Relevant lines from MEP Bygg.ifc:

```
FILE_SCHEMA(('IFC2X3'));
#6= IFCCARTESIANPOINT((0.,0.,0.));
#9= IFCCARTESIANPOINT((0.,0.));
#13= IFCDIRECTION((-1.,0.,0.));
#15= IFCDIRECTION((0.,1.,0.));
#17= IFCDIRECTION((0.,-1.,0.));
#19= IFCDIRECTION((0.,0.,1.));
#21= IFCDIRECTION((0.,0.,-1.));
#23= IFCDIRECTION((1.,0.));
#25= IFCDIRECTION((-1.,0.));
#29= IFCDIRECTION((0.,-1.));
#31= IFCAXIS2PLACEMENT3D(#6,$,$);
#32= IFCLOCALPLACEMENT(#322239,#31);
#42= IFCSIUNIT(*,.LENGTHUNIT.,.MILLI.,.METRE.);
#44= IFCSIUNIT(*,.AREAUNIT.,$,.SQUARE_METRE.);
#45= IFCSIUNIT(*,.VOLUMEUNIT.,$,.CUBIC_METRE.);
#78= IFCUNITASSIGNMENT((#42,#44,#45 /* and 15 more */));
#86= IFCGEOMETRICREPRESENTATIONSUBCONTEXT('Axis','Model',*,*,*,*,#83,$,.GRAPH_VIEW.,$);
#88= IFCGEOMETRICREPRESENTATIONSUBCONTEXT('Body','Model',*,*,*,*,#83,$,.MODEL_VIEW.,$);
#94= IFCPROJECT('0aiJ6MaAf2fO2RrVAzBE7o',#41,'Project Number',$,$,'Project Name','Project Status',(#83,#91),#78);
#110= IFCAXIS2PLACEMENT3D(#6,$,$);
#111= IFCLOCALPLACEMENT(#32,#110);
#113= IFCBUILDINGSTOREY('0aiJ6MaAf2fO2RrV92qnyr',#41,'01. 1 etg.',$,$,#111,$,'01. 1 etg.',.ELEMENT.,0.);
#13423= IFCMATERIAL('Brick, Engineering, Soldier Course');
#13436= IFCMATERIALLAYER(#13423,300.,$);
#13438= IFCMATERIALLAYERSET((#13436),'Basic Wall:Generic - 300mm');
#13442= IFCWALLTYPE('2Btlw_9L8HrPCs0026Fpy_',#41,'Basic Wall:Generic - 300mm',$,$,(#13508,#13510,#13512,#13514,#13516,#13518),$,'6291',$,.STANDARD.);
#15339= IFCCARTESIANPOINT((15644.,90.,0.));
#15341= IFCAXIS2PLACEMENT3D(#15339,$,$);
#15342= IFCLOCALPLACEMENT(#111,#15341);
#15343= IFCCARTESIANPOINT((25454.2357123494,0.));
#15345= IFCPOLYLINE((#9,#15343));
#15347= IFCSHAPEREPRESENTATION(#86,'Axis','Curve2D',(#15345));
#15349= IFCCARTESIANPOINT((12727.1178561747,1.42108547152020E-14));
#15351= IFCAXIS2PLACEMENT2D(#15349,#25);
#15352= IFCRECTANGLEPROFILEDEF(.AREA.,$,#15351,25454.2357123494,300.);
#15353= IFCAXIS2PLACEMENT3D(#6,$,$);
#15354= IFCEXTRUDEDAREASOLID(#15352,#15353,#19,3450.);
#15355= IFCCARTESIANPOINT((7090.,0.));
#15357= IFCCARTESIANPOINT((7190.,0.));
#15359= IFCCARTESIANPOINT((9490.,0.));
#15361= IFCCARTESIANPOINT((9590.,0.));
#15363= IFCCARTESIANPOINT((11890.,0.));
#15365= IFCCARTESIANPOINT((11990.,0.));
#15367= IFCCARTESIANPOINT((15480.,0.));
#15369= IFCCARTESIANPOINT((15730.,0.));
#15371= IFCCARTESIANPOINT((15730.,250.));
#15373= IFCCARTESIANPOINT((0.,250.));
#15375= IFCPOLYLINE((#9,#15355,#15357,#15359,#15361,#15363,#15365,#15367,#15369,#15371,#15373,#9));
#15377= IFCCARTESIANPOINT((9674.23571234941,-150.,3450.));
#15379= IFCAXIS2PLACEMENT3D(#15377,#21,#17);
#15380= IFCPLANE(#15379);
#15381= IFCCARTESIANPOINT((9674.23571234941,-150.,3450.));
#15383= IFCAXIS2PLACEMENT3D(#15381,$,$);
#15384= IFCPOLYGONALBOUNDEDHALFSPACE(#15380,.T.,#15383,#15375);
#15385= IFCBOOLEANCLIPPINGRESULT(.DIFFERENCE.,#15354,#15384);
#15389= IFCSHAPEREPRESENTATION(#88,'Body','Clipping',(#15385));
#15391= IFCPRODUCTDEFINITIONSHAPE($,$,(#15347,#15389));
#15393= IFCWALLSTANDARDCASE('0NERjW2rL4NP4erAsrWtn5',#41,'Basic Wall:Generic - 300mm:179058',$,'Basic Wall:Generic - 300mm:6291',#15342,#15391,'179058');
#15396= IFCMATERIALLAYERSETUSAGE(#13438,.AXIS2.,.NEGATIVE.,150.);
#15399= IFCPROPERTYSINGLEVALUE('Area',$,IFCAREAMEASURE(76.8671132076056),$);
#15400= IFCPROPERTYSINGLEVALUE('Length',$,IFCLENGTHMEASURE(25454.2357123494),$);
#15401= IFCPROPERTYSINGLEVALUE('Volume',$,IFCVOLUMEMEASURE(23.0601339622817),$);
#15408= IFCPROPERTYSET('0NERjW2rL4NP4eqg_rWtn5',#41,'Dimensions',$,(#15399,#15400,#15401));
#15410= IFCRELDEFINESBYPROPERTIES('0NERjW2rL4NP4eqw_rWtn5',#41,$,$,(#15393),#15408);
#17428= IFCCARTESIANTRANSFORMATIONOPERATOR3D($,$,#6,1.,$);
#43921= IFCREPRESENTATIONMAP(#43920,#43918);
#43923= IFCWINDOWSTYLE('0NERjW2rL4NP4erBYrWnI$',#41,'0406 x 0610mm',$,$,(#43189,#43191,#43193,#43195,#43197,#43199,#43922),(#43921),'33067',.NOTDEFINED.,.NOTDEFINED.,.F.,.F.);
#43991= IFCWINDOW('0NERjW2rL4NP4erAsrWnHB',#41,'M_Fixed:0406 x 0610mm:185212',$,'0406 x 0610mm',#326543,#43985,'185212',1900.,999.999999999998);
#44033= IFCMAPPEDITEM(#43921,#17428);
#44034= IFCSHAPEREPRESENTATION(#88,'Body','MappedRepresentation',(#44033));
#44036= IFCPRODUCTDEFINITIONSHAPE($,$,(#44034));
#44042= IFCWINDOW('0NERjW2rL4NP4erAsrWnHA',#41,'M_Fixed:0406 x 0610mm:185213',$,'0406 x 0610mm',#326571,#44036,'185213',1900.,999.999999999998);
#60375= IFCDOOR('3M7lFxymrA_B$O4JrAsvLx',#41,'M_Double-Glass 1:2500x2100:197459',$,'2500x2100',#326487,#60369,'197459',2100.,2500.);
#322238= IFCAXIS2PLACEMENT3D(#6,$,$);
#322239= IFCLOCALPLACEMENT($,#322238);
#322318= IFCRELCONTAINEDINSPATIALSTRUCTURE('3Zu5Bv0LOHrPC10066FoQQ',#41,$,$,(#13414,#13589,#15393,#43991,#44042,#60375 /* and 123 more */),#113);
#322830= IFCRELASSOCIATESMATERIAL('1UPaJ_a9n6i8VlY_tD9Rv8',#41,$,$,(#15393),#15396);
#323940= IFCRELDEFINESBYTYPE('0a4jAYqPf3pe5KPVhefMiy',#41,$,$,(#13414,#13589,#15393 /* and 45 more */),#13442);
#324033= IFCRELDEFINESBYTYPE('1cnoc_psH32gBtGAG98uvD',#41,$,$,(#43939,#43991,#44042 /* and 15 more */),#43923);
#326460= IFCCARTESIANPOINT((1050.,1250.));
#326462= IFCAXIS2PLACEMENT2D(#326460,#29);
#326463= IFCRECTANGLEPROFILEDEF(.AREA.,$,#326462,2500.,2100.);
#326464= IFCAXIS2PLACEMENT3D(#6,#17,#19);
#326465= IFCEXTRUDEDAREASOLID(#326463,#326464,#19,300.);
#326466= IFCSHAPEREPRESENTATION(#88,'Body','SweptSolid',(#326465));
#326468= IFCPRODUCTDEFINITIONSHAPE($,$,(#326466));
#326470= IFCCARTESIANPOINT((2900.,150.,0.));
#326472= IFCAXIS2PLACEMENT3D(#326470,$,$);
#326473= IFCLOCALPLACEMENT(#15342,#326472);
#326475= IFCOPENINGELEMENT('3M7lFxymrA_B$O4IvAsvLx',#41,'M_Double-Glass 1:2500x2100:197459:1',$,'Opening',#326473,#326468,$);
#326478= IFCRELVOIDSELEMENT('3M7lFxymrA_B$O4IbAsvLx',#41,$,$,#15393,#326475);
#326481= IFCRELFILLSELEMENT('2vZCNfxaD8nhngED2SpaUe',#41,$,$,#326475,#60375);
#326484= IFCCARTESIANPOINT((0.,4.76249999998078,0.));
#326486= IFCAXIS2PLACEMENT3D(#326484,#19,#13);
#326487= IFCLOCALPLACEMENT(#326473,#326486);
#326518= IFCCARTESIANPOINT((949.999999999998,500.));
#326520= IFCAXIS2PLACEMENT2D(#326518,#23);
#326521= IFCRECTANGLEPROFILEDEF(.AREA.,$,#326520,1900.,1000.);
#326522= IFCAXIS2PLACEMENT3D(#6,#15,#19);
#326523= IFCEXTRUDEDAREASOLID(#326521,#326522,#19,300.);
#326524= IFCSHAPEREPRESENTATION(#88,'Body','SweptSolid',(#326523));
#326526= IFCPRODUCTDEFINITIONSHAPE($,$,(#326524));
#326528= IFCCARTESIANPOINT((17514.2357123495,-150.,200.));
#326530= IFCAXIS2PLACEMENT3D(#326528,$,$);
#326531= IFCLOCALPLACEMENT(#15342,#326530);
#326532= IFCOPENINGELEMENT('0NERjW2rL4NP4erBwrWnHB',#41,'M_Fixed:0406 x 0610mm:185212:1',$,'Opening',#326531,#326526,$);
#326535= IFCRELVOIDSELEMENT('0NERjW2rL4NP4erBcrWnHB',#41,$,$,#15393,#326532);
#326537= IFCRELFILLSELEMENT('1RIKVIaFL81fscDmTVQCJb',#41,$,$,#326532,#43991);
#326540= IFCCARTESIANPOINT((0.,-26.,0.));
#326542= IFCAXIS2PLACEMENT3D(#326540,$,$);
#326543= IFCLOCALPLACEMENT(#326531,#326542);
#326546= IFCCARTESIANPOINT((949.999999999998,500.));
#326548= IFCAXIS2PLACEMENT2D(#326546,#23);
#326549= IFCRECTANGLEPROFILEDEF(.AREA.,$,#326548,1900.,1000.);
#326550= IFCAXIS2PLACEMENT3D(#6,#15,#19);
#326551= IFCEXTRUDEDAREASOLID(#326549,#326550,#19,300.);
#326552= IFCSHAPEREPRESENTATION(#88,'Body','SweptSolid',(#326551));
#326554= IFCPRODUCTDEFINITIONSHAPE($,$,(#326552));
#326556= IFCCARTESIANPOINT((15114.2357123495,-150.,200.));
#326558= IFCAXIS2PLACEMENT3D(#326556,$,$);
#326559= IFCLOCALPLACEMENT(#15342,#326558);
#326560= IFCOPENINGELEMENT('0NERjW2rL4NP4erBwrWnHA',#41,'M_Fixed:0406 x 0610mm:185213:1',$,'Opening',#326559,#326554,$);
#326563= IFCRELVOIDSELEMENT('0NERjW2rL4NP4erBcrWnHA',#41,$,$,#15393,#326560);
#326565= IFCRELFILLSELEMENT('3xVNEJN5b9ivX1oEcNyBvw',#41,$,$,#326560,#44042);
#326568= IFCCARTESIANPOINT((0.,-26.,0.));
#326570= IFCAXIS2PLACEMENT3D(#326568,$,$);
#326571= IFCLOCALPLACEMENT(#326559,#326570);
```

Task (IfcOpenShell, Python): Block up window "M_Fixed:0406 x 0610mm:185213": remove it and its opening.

```python
import ifcopenshell
import ifcopenshell.api.feature
import ifcopenshell.api.pset
import ifcopenshell.api.root
import ifcopenshell.geom
import ifcopenshell.util.element
import ifcopenshell.util.shape
import ifcopenshell.util.unit

model = ifcopenshell.open("MEP Bygg.ifc")
area_scale = ifcopenshell.util.unit.calculate_unit_scale(model, "AREAUNIT")
volume_scale = ifcopenshell.util.unit.calculate_unit_scale(model, "VOLUMEUNIT")
settings = ifcopenshell.geom.settings()


def volume(element):
    """Net volume in cubic metres, openings subtracted."""
    shape = ifcopenshell.geom.create_shape(settings, element)
    return ifcopenshell.util.shape.get_volume(shape.geometry)


window = model.by_guid("0NERjW2rL4NP4erAsrWnHA")
opening = window.FillsVoids[0].RelatingOpeningElement
wall = opening.VoidsElements[0].RelatingBuildingElement
before = volume(wall)

ifcopenshell.api.root.remove_product(model, product=window)
ifcopenshell.api.feature.remove_feature(model, feature=opening)

after = volume(wall)
thickness = 0.3  # wall thickness in metres

# Update the wall's stored quantities.
pset = model.by_id(ifcopenshell.util.element.get_pset(wall, "Dimensions", should_inherit=False)["id"])
ifcopenshell.api.pset.edit_pset(model, pset=pset, properties={
    "Area": model.create_entity("IfcAreaMeasure", after / thickness / area_scale),
    "Volume": model.create_entity("IfcVolumeMeasure", after / volume_scale),
})

print(f"wall volume {before:.3f} -> {after:.3f} m3")

model.write("MEP Bygg_edited.ifc")
```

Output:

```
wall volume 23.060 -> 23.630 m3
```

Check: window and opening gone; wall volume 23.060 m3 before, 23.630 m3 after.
